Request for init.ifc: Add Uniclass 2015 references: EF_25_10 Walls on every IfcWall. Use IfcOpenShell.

First a look at what the model holds.

```python
import ifcopenshell

model = ifcopenshell.open("init.ifc")
print(model.schema)
print("classifications:", [c.Name for c in model.by_type("IfcClassification")])
for ifc_class in ("IfcDoor", "IfcRoof", "IfcStair", "IfcWall", "IfcWindow"):
    print(ifc_class, len(model.by_type(ifc_class)))
```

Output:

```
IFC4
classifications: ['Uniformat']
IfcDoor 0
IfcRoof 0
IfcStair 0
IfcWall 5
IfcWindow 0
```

```python
import ifcopenshell
import ifcopenshell.api.classification

model = ifcopenshell.open("init.ifc")

system = ifcopenshell.api.classification.add_classification(model, classification="Uniclass 2015")

codes = {
    "IfcWall": ("EF_25_10", "Walls"),
}
for ifc_class, (code, name) in codes.items():
    products = model.by_type(ifc_class)
    ifcopenshell.api.classification.add_reference(
        model, products=products, classification=system, identification=code, name=name
    )
    print(code, len(products))

model.write("init_updated.ifc")
```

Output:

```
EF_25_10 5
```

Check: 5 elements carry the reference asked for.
